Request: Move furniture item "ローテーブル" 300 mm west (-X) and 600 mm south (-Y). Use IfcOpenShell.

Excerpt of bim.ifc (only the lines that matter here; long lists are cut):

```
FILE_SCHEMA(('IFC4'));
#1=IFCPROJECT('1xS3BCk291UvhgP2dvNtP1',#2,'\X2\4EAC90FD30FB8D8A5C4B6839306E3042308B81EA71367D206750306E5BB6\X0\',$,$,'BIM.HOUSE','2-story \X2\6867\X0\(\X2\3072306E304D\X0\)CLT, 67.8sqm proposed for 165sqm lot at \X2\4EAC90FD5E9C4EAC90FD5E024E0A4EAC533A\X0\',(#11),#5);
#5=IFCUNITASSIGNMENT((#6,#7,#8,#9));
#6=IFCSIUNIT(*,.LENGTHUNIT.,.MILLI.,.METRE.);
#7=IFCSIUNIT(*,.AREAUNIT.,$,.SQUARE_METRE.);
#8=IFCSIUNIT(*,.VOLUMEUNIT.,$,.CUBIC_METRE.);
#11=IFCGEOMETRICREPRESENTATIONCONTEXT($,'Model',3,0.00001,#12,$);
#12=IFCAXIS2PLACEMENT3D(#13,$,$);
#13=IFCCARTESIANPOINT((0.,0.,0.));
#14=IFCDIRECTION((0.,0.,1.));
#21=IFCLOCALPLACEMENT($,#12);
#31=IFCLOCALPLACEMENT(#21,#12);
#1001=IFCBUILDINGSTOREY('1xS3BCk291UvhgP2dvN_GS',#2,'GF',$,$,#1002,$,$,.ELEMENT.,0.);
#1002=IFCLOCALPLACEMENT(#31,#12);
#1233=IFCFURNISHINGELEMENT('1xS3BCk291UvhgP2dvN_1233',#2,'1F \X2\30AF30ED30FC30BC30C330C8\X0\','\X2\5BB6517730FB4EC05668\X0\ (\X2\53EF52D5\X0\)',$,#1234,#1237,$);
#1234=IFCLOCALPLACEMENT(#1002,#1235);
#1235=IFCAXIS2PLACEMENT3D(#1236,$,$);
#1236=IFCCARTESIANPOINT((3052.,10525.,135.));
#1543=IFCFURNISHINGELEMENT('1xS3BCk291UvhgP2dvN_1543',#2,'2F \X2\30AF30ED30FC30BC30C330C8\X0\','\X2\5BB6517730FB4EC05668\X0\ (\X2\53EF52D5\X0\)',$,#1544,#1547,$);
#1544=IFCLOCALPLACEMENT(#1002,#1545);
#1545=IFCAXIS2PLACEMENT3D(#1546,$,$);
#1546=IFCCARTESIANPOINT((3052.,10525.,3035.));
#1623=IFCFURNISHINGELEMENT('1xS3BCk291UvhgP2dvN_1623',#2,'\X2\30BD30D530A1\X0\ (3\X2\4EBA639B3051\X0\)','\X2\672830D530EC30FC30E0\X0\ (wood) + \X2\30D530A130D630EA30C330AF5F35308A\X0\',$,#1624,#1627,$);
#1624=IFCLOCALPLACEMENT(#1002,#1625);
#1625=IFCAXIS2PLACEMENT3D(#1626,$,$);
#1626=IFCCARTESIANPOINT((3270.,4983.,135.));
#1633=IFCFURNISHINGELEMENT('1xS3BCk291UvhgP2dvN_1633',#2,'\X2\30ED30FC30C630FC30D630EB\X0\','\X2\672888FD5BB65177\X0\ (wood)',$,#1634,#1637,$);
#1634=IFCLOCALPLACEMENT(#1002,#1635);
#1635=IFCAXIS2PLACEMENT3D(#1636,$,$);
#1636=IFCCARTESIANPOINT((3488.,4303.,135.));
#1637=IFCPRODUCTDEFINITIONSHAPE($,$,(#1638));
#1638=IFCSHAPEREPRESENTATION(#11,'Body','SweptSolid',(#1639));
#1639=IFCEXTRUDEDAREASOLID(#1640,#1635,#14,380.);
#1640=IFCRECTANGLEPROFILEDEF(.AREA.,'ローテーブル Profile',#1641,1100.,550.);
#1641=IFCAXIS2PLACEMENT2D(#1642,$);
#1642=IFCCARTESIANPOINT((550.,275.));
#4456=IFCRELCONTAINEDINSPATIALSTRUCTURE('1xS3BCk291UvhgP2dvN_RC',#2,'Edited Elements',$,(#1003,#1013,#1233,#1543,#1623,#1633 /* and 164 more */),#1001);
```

```python
import ifcopenshell
import ifcopenshell.api.geometry
import ifcopenshell.util.placement
import ifcopenshell.util.unit

model = ifcopenshell.open("bim.ifc")
unit_scale = ifcopenshell.util.unit.calculate_unit_scale(model)

item = model.by_guid("1xS3BCk291UvhgP2dvN_1633")
matrix = ifcopenshell.util.placement.get_local_placement(item.ObjectPlacement)
matrix[0, 3] -= 0.3 / unit_scale
matrix[1, 3] -= 0.6 / unit_scale
ifcopenshell.api.geometry.edit_object_placement(model, product=item, matrix=matrix, is_si=False)

print(ifcopenshell.util.placement.get_local_placement(item.ObjectPlacement).round(3) + 0.0)

model.write("bim_v2.ifc")
```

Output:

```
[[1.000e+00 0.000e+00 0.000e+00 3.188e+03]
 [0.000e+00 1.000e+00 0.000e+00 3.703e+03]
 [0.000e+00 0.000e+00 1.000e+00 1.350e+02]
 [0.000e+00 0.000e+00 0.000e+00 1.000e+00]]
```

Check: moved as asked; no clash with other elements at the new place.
